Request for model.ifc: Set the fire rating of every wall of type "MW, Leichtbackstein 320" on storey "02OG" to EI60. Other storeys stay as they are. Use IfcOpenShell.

First a look at what the model holds.

```python
import ifcopenshell
import ifcopenshell.util.element

model = ifcopenshell.open("model.ifc")
print(model.schema)
storey = next(s for s in model.by_type("IfcBuildingStorey") if s.Name == "02OG")
walls = [e for e in ifcopenshell.util.element.get_decomposition(storey) if e.is_a("IfcWall")]
seen = {}
for e in walls:
    element_type = ifcopenshell.util.element.get_type(e)
    key = (element_type.Name if element_type != e and element_type else None, ifcopenshell.util.element.get_pset(e, "Pset_WallCommon", "FireRating"))
    seen[key] = seen.get(key, 0) + 1
for (name, value), count in sorted(seen.items(), key=str):
    print(count, "x", name, "|", value)
```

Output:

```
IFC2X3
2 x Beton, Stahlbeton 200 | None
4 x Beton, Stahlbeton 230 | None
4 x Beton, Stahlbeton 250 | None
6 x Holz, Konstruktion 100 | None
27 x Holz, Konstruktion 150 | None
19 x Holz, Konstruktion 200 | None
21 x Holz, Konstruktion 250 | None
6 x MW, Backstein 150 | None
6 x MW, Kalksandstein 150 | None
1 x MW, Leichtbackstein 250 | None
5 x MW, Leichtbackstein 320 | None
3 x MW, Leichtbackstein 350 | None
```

```python
import ifcopenshell
import ifcopenshell.api.pset
import ifcopenshell.util.element

model = ifcopenshell.open("model.ifc")

storey = next(s for s in model.by_type("IfcBuildingStorey") if s.Name == "02OG")
walls = [e for e in ifcopenshell.util.element.get_decomposition(storey) if e.is_a("IfcWall")]

count = 0
for e in walls:
    element_type = ifcopenshell.util.element.get_type(e)
    if element_type in (None, e) or element_type.Name != "MW, Leichtbackstein 320":
        continue
    found = ifcopenshell.util.element.get_pset(e, "Pset_WallCommon", should_inherit=False)
    if found:
        pset = model.by_id(found["id"])
        if len(ifcopenshell.util.element.get_elements_by_pset(pset)) > 1:
            pset = ifcopenshell.api.pset.unshare_pset(model, products=[e], pset=pset)[0]
    else:
        pset = ifcopenshell.api.pset.add_pset(model, product=e, name="Pset_WallCommon")
    ifcopenshell.api.pset.edit_pset(model, pset=pset, properties={"FireRating": "EI60"})
    count += 1

print(count, "walls updated")

model.write("model_rev.ifc")
```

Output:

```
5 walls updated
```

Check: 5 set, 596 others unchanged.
